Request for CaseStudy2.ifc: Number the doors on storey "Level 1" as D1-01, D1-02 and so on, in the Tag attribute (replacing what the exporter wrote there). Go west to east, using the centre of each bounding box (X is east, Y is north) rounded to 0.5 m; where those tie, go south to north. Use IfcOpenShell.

First a look at what the model holds.

```python
import ifcopenshell
import ifcopenshell.util.element
import ifcopenshell.util.placement

model = ifcopenshell.open("CaseStudy2.ifc")
print(model.schema)
storey = next(s for s in model.by_type("IfcBuildingStorey") if s.Name == "Level 1")
doors = [e for e in ifcopenshell.util.element.get_decomposition(storey) if e.is_a("IfcDoor")]
for e in sorted(doors, key=lambda e: e.id()):
    origin = ifcopenshell.util.placement.get_local_placement(e.ObjectPlacement)[:3, 3]
    print(e.id(), e.Tag, e.Name, origin.round(2) + 0.0, sep=" | ")
```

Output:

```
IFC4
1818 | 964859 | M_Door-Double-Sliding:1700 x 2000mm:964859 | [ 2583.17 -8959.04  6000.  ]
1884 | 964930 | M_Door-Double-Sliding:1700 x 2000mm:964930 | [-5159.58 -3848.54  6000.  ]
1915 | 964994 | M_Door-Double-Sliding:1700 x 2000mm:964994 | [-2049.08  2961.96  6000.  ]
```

```python
import ifcopenshell
import ifcopenshell.geom
import ifcopenshell.util.element
import ifcopenshell.util.shape

model = ifcopenshell.open("CaseStudy2.ifc")
settings = ifcopenshell.geom.settings()
settings.set("use-world-coords", True)


def centre(element):
    shape = ifcopenshell.geom.create_shape(settings, element)
    return ifcopenshell.util.shape.get_bbox_centroid(shape.geometry)


storey = next(s for s in model.by_type("IfcBuildingStorey") if s.Name == "Level 1")
doors = [e for e in ifcopenshell.util.element.get_decomposition(storey) if e.is_a("IfcDoor")]

# Insertion points can sit at a corner or the storey origin, so sort by the geometry (in metres).
centres = {e: centre(e) for e in doors}
doors.sort(key=lambda e: (round(centres[e][0] / 0.5), centres[e][1]))

for i, e in enumerate(doors, start=1):
    number = f"D1-{i:02d}"
    e.Tag = number
    print(e.id(), number)

model.write("CaseStudy2-out.ifc")
```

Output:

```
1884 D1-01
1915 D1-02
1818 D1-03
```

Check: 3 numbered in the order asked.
